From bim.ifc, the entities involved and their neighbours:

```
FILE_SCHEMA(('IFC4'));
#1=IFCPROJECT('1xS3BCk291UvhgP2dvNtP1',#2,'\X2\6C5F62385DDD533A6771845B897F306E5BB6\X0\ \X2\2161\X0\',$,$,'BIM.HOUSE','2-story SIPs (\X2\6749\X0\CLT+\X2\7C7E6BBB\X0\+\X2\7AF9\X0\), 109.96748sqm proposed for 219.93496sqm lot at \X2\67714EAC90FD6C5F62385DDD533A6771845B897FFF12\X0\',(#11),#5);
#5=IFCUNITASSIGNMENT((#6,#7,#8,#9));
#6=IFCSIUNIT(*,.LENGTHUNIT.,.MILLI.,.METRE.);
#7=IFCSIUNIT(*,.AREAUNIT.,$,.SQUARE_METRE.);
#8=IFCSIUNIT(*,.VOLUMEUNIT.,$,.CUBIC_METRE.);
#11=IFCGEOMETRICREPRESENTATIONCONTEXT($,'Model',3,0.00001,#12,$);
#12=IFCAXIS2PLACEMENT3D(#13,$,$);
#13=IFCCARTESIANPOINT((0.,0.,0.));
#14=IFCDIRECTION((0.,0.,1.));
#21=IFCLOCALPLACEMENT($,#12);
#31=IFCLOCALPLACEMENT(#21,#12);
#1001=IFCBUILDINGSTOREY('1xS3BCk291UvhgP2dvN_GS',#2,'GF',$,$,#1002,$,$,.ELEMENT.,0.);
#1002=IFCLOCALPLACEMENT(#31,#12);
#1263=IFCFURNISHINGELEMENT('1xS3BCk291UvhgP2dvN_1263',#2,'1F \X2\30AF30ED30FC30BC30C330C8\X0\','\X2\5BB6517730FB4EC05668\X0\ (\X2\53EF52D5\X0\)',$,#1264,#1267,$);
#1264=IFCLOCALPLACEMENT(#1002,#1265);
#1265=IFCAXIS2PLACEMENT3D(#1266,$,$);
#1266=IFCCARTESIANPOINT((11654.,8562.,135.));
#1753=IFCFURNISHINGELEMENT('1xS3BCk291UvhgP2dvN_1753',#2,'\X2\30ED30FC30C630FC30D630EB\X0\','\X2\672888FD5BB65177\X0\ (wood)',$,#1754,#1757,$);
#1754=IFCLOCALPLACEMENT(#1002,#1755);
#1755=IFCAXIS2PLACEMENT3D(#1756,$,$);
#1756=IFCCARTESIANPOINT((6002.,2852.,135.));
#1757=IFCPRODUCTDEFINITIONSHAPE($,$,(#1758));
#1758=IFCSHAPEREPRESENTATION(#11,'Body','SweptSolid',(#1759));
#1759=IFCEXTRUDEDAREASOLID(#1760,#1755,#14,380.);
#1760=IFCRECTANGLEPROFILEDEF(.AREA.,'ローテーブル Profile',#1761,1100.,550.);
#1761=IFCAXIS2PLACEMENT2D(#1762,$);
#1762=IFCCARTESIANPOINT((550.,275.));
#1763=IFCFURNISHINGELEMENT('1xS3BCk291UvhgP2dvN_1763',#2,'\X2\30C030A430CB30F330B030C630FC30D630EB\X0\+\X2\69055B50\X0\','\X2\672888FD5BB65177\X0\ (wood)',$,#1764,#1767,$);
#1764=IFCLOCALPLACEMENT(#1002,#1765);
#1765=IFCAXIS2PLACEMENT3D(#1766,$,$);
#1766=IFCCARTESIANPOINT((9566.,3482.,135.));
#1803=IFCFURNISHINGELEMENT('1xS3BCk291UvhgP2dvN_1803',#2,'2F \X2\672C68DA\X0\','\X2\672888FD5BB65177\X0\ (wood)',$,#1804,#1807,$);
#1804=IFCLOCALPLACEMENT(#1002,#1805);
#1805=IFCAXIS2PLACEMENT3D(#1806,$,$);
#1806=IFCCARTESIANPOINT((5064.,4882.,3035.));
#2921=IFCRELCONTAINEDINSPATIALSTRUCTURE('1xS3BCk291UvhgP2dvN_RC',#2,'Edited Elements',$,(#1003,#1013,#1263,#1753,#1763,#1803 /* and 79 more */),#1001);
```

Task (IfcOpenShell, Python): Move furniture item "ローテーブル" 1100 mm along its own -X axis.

```python
import ifcopenshell
import ifcopenshell.api.geometry
import ifcopenshell.util.placement

model = ifcopenshell.open("bim.ifc")

item = model.by_id(1753)
matrix = ifcopenshell.util.placement.get_local_placement(item.ObjectPlacement)
matrix[:3, 3] -= matrix[:3, 0] * 1100.0
ifcopenshell.api.geometry.edit_object_placement(model, product=item, matrix=matrix, is_si=False)

print(ifcopenshell.util.placement.get_local_placement(item.ObjectPlacement).round(3) + 0.0)

model.write("bim_v2.ifc")
```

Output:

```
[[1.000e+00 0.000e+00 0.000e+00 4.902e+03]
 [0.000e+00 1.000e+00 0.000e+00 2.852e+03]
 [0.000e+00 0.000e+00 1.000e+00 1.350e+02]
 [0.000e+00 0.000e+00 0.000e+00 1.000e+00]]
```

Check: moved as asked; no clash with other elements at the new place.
